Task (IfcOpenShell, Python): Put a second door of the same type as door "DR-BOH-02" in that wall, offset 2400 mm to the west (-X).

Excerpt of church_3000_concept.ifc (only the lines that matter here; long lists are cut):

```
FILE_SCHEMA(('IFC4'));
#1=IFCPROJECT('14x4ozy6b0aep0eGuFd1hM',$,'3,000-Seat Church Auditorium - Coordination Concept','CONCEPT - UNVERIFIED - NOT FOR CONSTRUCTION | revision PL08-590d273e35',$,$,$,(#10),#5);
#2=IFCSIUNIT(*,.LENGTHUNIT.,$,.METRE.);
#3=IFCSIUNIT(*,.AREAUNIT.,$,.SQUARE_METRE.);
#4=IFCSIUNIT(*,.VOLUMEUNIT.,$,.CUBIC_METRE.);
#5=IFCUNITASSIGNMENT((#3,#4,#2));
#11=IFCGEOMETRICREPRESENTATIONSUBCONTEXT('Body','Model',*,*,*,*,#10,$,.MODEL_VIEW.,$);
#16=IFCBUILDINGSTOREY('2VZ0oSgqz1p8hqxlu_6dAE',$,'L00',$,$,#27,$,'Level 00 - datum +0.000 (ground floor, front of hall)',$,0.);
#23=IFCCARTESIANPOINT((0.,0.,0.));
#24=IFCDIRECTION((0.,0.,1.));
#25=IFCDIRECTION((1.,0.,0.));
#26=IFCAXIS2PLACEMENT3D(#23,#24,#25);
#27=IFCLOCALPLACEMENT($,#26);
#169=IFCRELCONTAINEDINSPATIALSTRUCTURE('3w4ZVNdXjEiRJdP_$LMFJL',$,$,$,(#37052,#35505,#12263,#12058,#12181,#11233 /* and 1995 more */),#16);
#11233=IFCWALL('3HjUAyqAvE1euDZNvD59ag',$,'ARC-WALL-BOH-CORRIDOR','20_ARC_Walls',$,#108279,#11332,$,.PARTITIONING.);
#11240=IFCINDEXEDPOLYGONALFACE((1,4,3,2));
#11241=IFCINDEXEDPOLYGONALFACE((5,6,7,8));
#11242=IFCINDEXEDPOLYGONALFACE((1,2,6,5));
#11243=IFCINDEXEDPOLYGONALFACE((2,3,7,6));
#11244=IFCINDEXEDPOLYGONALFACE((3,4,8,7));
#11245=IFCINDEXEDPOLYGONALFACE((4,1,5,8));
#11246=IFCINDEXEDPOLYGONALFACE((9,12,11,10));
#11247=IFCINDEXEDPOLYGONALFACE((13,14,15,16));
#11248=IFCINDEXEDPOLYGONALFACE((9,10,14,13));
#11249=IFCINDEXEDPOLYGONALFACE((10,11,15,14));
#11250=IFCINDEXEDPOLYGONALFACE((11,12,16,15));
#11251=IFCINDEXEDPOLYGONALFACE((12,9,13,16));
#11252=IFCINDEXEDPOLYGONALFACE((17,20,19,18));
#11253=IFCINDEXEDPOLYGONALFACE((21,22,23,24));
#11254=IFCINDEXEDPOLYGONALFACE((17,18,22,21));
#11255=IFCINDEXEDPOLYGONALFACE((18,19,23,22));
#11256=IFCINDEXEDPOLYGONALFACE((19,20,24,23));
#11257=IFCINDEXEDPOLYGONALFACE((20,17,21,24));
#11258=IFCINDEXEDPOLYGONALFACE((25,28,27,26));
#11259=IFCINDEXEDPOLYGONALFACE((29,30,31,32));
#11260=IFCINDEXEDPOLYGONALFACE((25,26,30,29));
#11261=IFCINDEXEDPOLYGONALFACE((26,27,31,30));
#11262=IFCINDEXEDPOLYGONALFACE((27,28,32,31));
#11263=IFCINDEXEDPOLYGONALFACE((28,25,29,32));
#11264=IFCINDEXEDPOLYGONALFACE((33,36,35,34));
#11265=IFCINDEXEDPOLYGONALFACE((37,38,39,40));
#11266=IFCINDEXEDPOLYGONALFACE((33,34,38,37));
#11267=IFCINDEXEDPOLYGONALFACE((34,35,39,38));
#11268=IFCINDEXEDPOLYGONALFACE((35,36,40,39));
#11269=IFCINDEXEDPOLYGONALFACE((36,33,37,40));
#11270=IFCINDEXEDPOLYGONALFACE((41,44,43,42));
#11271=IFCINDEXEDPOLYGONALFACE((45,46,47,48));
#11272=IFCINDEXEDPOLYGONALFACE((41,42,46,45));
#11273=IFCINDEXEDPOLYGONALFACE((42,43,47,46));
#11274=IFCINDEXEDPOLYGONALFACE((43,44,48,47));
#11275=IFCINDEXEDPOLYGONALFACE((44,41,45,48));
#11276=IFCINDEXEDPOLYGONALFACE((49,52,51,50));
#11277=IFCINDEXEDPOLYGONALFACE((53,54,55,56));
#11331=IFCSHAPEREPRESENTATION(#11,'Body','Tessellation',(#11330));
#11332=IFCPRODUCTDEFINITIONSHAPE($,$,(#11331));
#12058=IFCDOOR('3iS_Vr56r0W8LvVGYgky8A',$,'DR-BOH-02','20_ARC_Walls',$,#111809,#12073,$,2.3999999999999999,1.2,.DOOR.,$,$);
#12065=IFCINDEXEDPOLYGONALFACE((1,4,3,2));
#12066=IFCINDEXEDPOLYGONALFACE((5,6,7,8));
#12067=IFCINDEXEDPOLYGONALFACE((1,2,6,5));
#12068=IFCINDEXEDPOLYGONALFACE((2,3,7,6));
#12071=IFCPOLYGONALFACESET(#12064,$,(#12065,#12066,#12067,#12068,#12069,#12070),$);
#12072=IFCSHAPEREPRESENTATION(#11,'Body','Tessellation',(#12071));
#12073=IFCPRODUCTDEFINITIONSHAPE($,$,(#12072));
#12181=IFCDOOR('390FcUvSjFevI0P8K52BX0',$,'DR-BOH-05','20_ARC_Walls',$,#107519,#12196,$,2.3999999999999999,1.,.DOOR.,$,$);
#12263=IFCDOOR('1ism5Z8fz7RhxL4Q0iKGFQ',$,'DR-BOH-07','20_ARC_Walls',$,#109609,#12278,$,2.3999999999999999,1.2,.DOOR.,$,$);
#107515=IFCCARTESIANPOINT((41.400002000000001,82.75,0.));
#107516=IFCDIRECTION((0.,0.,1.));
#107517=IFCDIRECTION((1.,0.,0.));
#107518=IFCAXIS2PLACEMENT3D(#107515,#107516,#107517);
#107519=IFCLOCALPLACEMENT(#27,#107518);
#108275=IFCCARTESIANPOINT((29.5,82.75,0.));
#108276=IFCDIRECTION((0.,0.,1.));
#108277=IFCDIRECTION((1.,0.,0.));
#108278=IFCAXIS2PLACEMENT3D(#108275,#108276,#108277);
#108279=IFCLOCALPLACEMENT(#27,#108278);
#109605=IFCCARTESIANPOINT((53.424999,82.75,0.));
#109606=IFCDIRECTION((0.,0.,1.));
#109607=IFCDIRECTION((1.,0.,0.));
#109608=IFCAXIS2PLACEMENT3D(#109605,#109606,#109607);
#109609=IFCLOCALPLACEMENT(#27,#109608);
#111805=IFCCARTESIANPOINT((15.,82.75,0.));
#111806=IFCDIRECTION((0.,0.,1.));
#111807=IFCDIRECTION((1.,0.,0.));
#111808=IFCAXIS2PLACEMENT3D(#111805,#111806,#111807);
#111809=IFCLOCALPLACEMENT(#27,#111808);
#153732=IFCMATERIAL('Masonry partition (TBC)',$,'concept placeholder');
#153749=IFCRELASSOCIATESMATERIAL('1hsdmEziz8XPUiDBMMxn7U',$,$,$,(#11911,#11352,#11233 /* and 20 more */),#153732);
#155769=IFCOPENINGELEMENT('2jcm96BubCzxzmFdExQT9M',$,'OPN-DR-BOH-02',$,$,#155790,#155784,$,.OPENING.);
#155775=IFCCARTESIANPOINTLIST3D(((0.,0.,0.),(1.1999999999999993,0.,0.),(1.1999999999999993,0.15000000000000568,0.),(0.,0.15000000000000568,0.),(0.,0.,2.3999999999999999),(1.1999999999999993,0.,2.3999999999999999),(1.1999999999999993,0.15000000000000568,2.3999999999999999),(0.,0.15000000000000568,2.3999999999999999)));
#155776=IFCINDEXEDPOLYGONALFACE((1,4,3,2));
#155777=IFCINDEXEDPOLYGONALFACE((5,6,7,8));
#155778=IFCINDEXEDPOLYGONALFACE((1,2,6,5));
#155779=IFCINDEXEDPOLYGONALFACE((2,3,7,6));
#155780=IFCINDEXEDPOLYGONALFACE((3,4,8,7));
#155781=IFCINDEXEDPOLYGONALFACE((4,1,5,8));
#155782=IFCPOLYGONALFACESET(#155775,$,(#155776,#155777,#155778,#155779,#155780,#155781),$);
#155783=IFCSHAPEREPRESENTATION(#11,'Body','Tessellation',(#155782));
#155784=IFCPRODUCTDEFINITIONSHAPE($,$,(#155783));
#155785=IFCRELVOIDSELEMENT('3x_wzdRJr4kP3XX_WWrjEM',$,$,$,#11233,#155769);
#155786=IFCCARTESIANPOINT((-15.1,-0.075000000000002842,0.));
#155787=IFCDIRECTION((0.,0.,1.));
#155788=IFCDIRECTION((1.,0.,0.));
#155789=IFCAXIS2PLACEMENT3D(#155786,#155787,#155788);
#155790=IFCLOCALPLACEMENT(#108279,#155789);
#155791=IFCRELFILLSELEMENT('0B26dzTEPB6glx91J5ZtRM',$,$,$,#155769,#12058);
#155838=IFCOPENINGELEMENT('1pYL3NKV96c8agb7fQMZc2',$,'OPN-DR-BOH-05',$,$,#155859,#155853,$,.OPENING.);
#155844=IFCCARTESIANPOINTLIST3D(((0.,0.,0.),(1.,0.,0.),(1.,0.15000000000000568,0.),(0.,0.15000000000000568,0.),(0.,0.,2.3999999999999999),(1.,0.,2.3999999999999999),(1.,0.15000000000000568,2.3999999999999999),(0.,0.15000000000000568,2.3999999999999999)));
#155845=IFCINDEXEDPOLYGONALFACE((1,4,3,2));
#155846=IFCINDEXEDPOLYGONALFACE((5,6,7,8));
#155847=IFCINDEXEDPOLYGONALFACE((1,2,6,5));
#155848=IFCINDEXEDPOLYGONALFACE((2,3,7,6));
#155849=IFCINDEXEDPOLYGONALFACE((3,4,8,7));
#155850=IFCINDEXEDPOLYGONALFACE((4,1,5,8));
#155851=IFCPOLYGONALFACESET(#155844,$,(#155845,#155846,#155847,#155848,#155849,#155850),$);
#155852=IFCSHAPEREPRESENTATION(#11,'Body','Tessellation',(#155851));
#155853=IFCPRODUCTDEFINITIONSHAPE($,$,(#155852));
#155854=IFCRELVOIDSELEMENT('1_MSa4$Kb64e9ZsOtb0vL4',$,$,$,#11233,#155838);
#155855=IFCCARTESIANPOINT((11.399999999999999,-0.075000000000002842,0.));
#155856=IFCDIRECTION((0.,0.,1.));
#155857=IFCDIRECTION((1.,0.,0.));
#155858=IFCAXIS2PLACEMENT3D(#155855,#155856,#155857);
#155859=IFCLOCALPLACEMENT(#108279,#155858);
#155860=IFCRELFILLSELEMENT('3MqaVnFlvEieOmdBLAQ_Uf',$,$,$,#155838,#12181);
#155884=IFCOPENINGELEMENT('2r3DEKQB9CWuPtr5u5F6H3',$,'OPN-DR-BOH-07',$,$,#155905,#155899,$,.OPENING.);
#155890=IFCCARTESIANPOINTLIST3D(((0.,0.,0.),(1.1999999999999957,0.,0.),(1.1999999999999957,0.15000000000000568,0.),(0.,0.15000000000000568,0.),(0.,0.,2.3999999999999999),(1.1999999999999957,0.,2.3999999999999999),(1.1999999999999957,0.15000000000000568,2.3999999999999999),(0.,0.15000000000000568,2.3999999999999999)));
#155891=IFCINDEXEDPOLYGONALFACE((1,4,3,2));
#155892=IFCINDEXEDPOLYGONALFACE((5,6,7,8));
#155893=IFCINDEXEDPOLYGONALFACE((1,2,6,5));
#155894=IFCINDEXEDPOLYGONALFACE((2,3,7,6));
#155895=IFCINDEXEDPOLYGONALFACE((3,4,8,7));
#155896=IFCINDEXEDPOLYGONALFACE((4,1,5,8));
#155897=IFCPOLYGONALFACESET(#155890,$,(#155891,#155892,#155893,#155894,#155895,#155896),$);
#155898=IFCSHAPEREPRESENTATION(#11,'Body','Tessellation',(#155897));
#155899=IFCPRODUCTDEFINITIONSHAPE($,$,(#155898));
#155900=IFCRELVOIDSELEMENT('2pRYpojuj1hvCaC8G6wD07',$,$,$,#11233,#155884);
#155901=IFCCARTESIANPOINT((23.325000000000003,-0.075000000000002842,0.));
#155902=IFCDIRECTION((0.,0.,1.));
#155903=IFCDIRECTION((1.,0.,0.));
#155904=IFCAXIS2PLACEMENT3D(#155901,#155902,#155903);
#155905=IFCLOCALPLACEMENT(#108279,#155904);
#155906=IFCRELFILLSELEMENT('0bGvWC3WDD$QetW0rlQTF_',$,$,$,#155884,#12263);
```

```python
import ifcopenshell
import ifcopenshell.api.feature
import ifcopenshell.api.geometry
import ifcopenshell.api.root
import ifcopenshell.geom
import ifcopenshell.util.element
import ifcopenshell.util.placement
import ifcopenshell.util.shape
import ifcopenshell.util.unit

model = ifcopenshell.open("church_3000_concept.ifc")
unit_scale = ifcopenshell.util.unit.calculate_unit_scale(model)
settings = ifcopenshell.geom.settings()


def volume(element):
    """Net volume in cubic metres, openings subtracted."""
    shape = ifcopenshell.geom.create_shape(settings, element)
    return ifcopenshell.util.shape.get_volume(shape.geometry)


door = model.by_id(12058)
opening = door.FillsVoids[0].RelatingOpeningElement
wall = opening.VoidsElements[0].RelatingBuildingElement
before = volume(wall)
shift = ifcopenshell.util.placement.get_local_placement(wall.ObjectPlacement)[:3, 0] * -2.4 / unit_scale

# copy_class copies the void relationship, type, container and properties, but no geometry.
new_opening = ifcopenshell.api.root.copy_class(model, product=opening)
new_opening.Representation = ifcopenshell.util.element.copy_deep(
    model, opening.Representation, exclude=["IfcGeometricRepresentationContext", "IfcRepresentationMap"]
)
new_door = ifcopenshell.api.root.copy_class(model, product=door)
new_door.Representation = ifcopenshell.util.element.copy_deep(
    model, door.Representation, exclude=["IfcGeometricRepresentationContext", "IfcRepresentationMap"]
)
ifcopenshell.api.feature.add_filling(model, opening=new_opening, element=new_door)

for old, new in ((opening, new_opening), (door, new_door)):
    matrix = ifcopenshell.util.placement.get_local_placement(old.ObjectPlacement)
    matrix[:3, 3] += shift
    ifcopenshell.api.geometry.edit_object_placement(model, product=new, matrix=matrix, is_si=False)

after = volume(wall)

print(f"wall volume {before:.3f} -> {after:.3f} m3")

model.write("church_3000_concept_edited.ifc")
```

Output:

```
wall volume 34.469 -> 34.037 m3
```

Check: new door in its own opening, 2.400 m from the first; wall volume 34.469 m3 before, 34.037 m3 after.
